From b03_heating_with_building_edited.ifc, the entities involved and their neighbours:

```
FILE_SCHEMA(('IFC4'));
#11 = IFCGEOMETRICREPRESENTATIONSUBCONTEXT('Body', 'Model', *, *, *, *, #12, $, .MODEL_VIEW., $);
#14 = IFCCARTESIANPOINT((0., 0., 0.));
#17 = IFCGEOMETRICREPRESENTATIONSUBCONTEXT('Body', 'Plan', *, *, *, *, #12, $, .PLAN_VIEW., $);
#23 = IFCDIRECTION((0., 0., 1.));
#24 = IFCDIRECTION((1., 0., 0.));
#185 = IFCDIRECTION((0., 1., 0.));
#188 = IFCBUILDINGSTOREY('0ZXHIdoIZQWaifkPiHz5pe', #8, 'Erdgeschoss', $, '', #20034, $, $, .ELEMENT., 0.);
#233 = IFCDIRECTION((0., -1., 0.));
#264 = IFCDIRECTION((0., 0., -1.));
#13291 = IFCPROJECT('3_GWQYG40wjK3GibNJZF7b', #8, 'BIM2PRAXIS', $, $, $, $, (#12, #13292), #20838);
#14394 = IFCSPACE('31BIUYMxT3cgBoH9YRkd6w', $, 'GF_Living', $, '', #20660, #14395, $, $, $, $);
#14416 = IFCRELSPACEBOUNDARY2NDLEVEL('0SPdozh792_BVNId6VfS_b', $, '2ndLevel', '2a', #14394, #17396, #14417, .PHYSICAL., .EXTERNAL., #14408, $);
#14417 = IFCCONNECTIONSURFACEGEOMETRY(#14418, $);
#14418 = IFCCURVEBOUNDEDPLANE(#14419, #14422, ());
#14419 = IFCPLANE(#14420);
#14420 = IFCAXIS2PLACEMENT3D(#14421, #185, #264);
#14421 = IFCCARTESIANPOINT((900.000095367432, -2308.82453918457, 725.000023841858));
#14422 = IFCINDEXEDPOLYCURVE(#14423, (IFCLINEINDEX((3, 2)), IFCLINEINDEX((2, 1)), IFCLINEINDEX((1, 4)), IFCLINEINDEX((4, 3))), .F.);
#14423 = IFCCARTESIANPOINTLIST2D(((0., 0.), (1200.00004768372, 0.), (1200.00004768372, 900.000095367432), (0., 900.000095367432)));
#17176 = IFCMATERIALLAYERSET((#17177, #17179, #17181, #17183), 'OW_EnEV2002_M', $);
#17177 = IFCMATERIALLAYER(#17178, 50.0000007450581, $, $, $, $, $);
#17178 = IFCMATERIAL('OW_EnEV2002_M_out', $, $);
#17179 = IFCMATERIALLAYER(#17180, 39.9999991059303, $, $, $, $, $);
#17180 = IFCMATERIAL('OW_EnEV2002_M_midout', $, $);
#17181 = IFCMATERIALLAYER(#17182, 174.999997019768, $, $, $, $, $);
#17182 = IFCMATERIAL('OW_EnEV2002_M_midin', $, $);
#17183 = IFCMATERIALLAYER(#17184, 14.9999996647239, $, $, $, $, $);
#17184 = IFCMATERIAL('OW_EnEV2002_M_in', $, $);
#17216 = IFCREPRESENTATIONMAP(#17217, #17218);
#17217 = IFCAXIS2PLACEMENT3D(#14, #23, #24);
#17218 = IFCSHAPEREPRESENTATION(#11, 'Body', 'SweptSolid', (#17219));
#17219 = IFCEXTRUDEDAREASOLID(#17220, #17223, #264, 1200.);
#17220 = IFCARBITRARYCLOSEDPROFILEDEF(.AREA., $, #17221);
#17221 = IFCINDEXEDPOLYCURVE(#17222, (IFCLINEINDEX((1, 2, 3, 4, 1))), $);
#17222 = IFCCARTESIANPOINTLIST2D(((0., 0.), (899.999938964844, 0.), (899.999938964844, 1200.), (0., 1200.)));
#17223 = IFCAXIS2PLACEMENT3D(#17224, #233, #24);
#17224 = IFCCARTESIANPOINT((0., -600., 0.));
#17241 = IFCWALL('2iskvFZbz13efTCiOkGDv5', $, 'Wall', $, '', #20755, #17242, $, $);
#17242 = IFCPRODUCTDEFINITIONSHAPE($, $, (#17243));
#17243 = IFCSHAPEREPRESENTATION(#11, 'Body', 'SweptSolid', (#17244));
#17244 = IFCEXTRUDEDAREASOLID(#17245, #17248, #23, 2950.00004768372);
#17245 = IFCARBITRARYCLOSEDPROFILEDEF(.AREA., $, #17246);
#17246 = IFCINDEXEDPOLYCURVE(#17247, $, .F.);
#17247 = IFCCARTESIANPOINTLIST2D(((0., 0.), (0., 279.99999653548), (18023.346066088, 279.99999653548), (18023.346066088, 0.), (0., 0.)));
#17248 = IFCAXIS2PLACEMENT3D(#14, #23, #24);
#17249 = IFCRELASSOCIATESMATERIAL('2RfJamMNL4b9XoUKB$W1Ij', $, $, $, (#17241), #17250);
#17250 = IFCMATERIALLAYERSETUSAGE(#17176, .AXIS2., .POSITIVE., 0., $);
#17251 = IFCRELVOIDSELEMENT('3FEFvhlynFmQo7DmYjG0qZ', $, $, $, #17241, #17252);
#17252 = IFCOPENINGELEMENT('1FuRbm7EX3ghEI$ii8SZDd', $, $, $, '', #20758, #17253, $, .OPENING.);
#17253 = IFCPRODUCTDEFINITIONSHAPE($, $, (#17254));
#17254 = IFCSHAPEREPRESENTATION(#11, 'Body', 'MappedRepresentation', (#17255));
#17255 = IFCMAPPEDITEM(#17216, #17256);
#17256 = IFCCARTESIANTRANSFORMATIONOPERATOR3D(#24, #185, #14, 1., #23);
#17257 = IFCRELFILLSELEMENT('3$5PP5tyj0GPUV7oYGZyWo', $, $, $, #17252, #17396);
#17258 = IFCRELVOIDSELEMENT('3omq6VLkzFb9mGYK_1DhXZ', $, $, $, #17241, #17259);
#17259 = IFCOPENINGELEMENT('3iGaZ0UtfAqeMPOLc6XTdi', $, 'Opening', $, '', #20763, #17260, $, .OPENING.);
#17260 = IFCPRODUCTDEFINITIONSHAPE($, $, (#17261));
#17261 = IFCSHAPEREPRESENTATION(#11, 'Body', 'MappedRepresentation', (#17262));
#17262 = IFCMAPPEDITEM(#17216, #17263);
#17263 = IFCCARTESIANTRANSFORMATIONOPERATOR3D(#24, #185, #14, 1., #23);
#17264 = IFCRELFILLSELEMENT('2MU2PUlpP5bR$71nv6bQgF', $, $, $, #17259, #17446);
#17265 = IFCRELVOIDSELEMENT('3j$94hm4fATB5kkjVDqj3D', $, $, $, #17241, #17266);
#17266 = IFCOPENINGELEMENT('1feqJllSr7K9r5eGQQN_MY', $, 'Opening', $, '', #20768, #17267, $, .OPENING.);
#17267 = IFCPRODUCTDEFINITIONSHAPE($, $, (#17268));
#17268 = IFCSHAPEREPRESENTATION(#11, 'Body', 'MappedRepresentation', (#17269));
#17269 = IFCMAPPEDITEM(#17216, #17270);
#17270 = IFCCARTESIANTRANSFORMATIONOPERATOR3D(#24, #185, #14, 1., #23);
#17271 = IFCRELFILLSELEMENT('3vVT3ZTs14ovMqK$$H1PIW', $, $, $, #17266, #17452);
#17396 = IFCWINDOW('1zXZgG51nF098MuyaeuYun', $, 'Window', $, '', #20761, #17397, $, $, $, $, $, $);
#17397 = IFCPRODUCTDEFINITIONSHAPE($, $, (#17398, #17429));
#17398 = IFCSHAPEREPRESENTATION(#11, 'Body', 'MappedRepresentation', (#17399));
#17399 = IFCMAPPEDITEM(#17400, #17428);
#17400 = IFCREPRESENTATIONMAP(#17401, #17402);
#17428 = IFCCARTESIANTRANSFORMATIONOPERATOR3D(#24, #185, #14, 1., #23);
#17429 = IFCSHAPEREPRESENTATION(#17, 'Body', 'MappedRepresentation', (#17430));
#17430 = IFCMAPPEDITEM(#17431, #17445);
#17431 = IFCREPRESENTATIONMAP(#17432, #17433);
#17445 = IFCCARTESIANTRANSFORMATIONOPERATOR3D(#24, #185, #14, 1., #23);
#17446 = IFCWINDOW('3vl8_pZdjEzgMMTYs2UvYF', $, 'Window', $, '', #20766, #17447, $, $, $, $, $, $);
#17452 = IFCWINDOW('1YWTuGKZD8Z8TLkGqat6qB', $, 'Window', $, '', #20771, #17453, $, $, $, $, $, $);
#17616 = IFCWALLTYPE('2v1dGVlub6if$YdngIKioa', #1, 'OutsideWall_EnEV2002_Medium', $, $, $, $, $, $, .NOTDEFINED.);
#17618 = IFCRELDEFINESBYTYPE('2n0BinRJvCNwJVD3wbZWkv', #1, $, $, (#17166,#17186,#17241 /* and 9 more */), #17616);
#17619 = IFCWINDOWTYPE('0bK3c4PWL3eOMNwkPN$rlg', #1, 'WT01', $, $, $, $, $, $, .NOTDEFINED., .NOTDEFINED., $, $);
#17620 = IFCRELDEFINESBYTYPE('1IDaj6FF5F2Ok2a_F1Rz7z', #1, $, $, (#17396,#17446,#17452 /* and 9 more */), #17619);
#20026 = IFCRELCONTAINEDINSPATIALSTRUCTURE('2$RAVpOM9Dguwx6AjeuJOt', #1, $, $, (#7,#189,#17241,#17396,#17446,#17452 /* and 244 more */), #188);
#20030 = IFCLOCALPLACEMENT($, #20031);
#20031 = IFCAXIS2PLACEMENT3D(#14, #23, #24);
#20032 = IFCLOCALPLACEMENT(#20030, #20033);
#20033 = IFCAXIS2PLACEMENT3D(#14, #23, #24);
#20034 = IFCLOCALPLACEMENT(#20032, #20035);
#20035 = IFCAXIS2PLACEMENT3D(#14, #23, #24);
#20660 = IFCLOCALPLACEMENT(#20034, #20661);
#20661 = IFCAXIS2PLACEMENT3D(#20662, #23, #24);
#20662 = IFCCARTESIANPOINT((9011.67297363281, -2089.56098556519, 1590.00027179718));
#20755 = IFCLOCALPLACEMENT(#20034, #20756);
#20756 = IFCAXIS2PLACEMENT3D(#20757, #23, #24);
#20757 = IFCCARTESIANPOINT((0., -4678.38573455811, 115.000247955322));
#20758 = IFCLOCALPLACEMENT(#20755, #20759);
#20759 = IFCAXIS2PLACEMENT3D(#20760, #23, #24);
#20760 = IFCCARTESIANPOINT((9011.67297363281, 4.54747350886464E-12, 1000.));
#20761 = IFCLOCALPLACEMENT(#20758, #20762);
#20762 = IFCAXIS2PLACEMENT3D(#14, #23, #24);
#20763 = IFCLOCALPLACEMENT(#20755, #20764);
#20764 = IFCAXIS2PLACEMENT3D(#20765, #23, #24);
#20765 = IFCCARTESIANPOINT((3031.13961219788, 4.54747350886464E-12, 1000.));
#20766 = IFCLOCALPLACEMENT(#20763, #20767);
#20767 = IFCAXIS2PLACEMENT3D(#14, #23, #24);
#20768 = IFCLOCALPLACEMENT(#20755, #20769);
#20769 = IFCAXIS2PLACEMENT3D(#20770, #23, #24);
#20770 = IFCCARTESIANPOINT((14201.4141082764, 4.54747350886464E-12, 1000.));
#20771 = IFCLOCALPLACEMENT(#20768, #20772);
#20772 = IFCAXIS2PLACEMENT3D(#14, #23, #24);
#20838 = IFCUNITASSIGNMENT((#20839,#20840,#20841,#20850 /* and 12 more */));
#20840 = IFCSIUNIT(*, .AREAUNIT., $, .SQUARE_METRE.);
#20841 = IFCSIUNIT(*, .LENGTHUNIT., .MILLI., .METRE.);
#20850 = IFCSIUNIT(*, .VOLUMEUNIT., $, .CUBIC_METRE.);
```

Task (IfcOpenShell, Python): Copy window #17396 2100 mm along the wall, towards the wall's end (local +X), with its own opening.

```python
import numpy as np
import ifcopenshell
import ifcopenshell.api.feature
import ifcopenshell.api.geometry
import ifcopenshell.api.root
import ifcopenshell.geom
import ifcopenshell.util.element
import ifcopenshell.util.placement
import ifcopenshell.util.shape
import ifcopenshell.util.unit

model = ifcopenshell.open("b03_heating_with_building_edited.ifc")
unit_scale = ifcopenshell.util.unit.calculate_unit_scale(model)
settings = ifcopenshell.geom.settings()


def volume(element):
    """Net volume in cubic metres, openings subtracted."""
    shape = ifcopenshell.geom.create_shape(settings, element)
    return ifcopenshell.util.shape.get_volume(shape.geometry)


def reuse_history(source, copy):
    """copy_class also copies each property set's owner history, people and application; keep the originals."""
    for rel in copy.IsDefinedBy:
        if rel.is_a("IfcRelDefinesByProperties") and (history := rel.RelatingPropertyDefinition.OwnerHistory):
            rel.RelatingPropertyDefinition.OwnerHistory = source.OwnerHistory
            ifcopenshell.util.element.remove_deep2(model, history)


window = model.by_guid("1zXZgG51nF098MuyaeuYun")
opening = window.FillsVoids[0].RelatingOpeningElement
wall = opening.VoidsElements[0].RelatingBuildingElement
before = volume(wall)
shift = ifcopenshell.util.placement.get_local_placement(wall.ObjectPlacement)[:3, 0] * 2.1 / unit_scale

# copy_class copies the void relationship, type, container and properties, but no geometry.
new_opening = ifcopenshell.api.root.copy_class(model, product=opening)
new_opening.Representation = ifcopenshell.util.element.copy_deep(
    model, opening.Representation, exclude=["IfcGeometricRepresentationContext", "IfcRepresentationMap"]
)
reuse_history(opening, new_opening)
new_window = ifcopenshell.api.root.copy_class(model, product=window)
new_window.Representation = ifcopenshell.util.element.copy_deep(
    model, window.Representation, exclude=["IfcGeometricRepresentationContext", "IfcRepresentationMap"]
)
reuse_history(window, new_window)
ifcopenshell.api.feature.add_filling(model, opening=new_opening, element=new_window)

for old, new in ((opening, new_opening), (window, new_window)):
    matrix = ifcopenshell.util.placement.get_local_placement(old.ObjectPlacement)
    matrix[:3, 3] += shift
    ifcopenshell.api.geometry.edit_object_placement(model, product=new, matrix=matrix, is_si=False)

# The copied space boundaries still share their surfaces with the original.
for rel in new_window.ProvidesBoundaries:
    if rel.ConnectionGeometry:
        rel.ConnectionGeometry = ifcopenshell.util.element.copy_deep(model, rel.ConnectionGeometry)

# Space boundary surfaces are stored in each space's coordinates; move them too.
for rel in new_window.ProvidesBoundaries:
    if not rel.ConnectionGeometry:
        continue
    surface = rel.ConnectionGeometry.SurfaceOnRelatingElement.BasisSurface
    space_matrix = ifcopenshell.util.placement.get_local_placement(rel.RelatingSpace.ObjectPlacement)
    point = np.array(surface.Position.Location.Coordinates) + space_matrix[:3, :3].T @ shift
    surface.Position = model.createIfcAxis2Placement3D(
        model.createIfcCartesianPoint(point.tolist()), surface.Position.Axis, surface.Position.RefDirection
    )

after = volume(wall)

print(f"wall volume {before:.3f} -> {after:.3f} m3")

model.write("b03_heating_with_building_edited-out.ifc")
```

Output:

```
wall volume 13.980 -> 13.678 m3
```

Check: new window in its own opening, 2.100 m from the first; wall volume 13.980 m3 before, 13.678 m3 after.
